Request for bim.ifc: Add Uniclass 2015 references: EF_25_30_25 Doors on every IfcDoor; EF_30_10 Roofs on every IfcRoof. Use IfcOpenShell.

First a look at what the model holds.

```python
import ifcopenshell

model = ifcopenshell.open("bim.ifc")
print(model.schema)
print("classifications:", [c.Name for c in model.by_type("IfcClassification")])
for ifc_class in ("IfcDoor", "IfcRoof", "IfcStair", "IfcWall", "IfcWindow"):
    print(ifc_class, len(model.by_type(ifc_class)))
```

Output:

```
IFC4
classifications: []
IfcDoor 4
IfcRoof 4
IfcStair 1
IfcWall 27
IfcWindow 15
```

```python
import ifcopenshell
import ifcopenshell.api.classification

model = ifcopenshell.open("bim.ifc")

system = ifcopenshell.api.classification.add_classification(model, classification="Uniclass 2015")

codes = {
    "IfcDoor": ("EF_25_30_25", "Doors"),
    "IfcRoof": ("EF_30_10", "Roofs"),
}
for ifc_class, (code, name) in codes.items():
    products = model.by_type(ifc_class)
    ifcopenshell.api.classification.add_reference(
        model, products=products, classification=system, identification=code, name=name
    )
    print(code, len(products))

model.write("bim_rev.ifc")
```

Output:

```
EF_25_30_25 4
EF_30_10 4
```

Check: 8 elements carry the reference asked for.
